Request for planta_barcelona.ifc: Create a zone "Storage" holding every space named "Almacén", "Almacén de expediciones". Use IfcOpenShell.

First a look at what the model holds.

```python
import ifcopenshell

model = ifcopenshell.open("planta_barcelona.ifc")
print(model.schema)
seen = {}
for space in model.by_type("IfcSpace"):
    seen[space.LongName] = seen.get(space.LongName, 0) + 1
for name, count in sorted(seen.items(), key=str):
    print(count, "x", name)
print("zones:", [z.Name for z in model.by_type("IfcZone")][:20])
```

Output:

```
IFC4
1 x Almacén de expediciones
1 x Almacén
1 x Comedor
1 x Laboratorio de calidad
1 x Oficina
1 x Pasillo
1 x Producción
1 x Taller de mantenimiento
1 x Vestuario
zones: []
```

```python
import ifcopenshell
import ifcopenshell.api.group
import ifcopenshell.api.root

model = ifcopenshell.open("planta_barcelona.ifc")

names = {"Almacén", "Almacén de expediciones"}
spaces = [s for s in model.by_type("IfcSpace") if s.LongName in names]

zone = ifcopenshell.api.root.create_entity(model, ifc_class="IfcZone", name="Storage")
ifcopenshell.api.group.assign_group(model, products=spaces, group=zone)
print(len(spaces), "spaces in", zone.Name)

model.write("planta_barcelona_rev.ifc")
```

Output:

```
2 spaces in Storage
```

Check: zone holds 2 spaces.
